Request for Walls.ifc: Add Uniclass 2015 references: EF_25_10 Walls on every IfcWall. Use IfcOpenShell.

First a look at what the model holds.

```python
import ifcopenshell

model = ifcopenshell.open("Walls.ifc")
print(model.schema)
print("classifications:", [c.Name for c in model.by_type("IfcClassification")])
for ifc_class in ("IfcDoor", "IfcRoof", "IfcStair", "IfcWall", "IfcWindow"):
    print(ifc_class, len(model.by_type(ifc_class)))
```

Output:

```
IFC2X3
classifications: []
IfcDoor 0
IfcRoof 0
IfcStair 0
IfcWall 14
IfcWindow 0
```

```python
import ifcopenshell
import ifcopenshell.api.classification

model = ifcopenshell.open("Walls.ifc")

# IFC2X3 requires Source and Edition and has no link from the project to the system.
system = model.create_entity("IfcClassification", Source="NBS", Edition="2015", Name="Uniclass 2015")

codes = {
    "IfcWall": ("EF_25_10", "Walls"),
}
for ifc_class, (code, name) in codes.items():
    products = model.by_type(ifc_class)
    ifcopenshell.api.classification.add_reference(
        model, products=products, classification=system, identification=code, name=name
    )
    print(code, len(products))

model.write("Walls-out.ifc")
```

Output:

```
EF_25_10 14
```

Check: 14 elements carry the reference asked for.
